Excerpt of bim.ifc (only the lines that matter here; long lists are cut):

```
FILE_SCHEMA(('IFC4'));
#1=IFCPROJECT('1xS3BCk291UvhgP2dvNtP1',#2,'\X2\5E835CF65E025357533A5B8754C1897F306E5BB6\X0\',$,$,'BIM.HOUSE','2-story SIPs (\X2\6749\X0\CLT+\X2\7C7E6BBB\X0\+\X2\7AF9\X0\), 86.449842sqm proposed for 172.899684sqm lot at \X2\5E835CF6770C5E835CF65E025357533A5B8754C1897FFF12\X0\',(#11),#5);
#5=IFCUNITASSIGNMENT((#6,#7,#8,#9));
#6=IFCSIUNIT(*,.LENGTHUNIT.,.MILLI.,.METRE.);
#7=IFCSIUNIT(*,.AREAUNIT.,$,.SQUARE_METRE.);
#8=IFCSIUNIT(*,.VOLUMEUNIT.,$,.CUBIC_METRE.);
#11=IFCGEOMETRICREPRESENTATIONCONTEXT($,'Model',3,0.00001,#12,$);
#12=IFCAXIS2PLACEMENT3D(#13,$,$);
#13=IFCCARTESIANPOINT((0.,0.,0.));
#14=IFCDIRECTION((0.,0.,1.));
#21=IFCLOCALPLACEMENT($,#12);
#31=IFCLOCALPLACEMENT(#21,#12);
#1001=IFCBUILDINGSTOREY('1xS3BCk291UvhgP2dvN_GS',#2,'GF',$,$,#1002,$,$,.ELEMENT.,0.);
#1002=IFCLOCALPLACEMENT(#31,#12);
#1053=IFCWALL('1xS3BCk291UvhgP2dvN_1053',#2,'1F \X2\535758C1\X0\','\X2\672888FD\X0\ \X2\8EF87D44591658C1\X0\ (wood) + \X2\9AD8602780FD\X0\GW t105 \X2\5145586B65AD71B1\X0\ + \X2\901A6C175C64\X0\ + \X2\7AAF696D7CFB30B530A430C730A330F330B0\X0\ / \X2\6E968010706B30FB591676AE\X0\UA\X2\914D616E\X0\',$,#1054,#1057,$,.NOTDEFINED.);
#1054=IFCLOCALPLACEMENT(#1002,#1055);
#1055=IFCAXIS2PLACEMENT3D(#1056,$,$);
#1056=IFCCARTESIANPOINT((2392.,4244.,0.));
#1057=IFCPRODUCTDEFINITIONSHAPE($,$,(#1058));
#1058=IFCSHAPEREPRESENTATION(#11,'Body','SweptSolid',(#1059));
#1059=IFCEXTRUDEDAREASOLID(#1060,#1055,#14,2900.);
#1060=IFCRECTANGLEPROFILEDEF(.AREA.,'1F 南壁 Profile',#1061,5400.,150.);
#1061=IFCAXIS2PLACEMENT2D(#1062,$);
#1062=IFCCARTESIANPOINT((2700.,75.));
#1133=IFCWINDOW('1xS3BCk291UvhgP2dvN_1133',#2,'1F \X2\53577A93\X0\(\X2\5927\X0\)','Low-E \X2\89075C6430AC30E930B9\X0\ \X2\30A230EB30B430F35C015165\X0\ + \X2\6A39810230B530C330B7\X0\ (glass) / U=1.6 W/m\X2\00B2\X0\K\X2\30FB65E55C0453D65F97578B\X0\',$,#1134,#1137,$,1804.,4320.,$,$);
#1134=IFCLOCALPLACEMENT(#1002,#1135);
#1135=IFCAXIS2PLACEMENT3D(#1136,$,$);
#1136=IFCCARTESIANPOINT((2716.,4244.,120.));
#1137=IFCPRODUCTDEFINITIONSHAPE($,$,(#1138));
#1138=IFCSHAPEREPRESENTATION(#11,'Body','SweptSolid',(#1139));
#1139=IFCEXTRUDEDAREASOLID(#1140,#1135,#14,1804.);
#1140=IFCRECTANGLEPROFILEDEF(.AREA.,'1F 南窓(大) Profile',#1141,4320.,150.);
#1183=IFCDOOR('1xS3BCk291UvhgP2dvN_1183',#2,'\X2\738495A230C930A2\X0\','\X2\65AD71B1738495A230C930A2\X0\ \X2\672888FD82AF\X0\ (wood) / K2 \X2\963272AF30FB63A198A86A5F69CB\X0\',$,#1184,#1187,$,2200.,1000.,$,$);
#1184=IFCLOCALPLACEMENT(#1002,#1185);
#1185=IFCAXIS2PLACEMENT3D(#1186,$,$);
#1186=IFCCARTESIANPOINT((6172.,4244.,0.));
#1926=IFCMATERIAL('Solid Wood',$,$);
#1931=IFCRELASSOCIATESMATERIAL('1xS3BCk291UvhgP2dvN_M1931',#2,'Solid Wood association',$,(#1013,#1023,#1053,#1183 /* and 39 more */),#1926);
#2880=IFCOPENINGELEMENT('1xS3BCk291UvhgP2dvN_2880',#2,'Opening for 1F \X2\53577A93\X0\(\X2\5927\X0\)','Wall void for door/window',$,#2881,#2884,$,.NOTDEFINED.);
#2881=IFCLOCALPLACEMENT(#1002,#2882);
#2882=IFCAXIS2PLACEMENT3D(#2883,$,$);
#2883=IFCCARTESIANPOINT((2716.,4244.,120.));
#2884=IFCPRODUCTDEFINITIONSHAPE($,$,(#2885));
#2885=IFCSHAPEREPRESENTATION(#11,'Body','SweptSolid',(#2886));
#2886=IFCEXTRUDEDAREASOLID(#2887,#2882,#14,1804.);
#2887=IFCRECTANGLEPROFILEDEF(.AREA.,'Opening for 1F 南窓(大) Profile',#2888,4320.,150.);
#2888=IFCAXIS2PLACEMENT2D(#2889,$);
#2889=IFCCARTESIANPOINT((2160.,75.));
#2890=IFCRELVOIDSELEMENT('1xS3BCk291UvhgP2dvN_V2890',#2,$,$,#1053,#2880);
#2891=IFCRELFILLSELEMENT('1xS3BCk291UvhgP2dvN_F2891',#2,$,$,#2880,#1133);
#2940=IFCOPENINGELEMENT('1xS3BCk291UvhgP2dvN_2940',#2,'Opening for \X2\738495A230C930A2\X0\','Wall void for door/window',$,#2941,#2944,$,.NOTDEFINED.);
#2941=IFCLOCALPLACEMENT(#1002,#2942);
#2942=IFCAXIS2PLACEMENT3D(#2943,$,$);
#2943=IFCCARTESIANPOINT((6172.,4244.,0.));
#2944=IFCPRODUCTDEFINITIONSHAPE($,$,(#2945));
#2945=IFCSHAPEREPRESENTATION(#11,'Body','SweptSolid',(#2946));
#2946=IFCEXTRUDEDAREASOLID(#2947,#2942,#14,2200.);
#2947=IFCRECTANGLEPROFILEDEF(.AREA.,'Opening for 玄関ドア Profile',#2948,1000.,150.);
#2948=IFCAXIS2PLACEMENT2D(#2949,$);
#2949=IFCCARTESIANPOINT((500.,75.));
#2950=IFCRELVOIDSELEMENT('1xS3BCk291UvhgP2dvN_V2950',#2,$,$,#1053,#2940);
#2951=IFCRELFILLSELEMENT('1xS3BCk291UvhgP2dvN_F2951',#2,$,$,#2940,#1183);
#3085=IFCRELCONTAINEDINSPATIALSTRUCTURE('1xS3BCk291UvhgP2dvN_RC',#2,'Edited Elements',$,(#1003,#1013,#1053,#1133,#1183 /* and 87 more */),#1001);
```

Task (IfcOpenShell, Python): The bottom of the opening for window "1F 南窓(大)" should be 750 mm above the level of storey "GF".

```python
import numpy as np
import ifcopenshell
import ifcopenshell.api.geometry
import ifcopenshell.geom
import ifcopenshell.util.element
import ifcopenshell.util.placement
import ifcopenshell.util.shape
import ifcopenshell.util.unit

model = ifcopenshell.open("bim.ifc")
unit_scale = ifcopenshell.util.unit.calculate_unit_scale(model)

window = model.by_id(1133)
opening = window.FillsVoids[0].RelatingOpeningElement
storey = ifcopenshell.util.element.get_container(window, ifc_class="IfcBuildingStorey")
level = ifcopenshell.util.placement.get_local_placement(storey.ObjectPlacement)[2, 3]

# The opening's origin need not be at the sill, so measure its lowest point.
shape = ifcopenshell.geom.create_shape(ifcopenshell.geom.settings(), opening)
bottom = ifcopenshell.util.shape.get_shape_bottom_elevation(shape, shape.geometry) / unit_scale
dz = level + 0.75 / unit_scale - bottom

shift = np.array([0.0, 0.0, dz])
# The window is not placed relative to its opening, so move both.
for product in (opening, window):
    matrix = ifcopenshell.util.placement.get_local_placement(product.ObjectPlacement)
    matrix[:3, 3] += shift
    ifcopenshell.api.geometry.edit_object_placement(model, product=product, matrix=matrix, is_si=False)

print(f"moved by {dz * unit_scale:+.3f} m")

model.write("bim_edited.ifc")
```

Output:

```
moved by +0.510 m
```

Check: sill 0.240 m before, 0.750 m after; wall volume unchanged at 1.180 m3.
